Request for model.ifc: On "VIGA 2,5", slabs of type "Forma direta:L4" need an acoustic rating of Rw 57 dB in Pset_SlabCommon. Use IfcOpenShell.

First a look at what the model holds.

```python
import ifcopenshell
import ifcopenshell.util.element

model = ifcopenshell.open("model.ifc")
print(model.schema)
storey = next(s for s in model.by_type("IfcBuildingStorey") if s.Name == "VIGA 2,5")
slabs = [e for e in ifcopenshell.util.element.get_decomposition(storey) if e.is_a("IfcSlab")]
seen = {}
for e in slabs:
    element_type = ifcopenshell.util.element.get_type(e)
    key = (element_type.Name if element_type != e and element_type else None, ifcopenshell.util.element.get_pset(e, "Pset_SlabCommon", "AcousticRating"))
    seen[key] = seen.get(key, 0) + 1
for (name, value), count in sorted(seen.items(), key=str):
    print(count, "x", name, "|", value)
```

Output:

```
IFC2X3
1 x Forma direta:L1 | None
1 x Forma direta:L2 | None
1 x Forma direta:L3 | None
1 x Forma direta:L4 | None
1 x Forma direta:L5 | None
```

```python
import ifcopenshell
import ifcopenshell.api.pset
import ifcopenshell.util.element

model = ifcopenshell.open("model.ifc")

storey = next(s for s in model.by_type("IfcBuildingStorey") if s.Name == "VIGA 2,5")
slabs = [e for e in ifcopenshell.util.element.get_decomposition(storey) if e.is_a("IfcSlab")]

count = 0
for e in slabs:
    element_type = ifcopenshell.util.element.get_type(e)
    if element_type in (None, e) or element_type.Name != "Forma direta:L4":
        continue
    # add_pset returns the element's existing set when there is one.
    pset = ifcopenshell.api.pset.add_pset(model, product=e, name="Pset_SlabCommon")
    ifcopenshell.api.pset.edit_pset(model, pset=pset, properties={"AcousticRating": "Rw 57 dB"})
    count += 1

print(count, "slabs updated")

model.write("model_v2.ifc")
```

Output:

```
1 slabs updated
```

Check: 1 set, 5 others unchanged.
